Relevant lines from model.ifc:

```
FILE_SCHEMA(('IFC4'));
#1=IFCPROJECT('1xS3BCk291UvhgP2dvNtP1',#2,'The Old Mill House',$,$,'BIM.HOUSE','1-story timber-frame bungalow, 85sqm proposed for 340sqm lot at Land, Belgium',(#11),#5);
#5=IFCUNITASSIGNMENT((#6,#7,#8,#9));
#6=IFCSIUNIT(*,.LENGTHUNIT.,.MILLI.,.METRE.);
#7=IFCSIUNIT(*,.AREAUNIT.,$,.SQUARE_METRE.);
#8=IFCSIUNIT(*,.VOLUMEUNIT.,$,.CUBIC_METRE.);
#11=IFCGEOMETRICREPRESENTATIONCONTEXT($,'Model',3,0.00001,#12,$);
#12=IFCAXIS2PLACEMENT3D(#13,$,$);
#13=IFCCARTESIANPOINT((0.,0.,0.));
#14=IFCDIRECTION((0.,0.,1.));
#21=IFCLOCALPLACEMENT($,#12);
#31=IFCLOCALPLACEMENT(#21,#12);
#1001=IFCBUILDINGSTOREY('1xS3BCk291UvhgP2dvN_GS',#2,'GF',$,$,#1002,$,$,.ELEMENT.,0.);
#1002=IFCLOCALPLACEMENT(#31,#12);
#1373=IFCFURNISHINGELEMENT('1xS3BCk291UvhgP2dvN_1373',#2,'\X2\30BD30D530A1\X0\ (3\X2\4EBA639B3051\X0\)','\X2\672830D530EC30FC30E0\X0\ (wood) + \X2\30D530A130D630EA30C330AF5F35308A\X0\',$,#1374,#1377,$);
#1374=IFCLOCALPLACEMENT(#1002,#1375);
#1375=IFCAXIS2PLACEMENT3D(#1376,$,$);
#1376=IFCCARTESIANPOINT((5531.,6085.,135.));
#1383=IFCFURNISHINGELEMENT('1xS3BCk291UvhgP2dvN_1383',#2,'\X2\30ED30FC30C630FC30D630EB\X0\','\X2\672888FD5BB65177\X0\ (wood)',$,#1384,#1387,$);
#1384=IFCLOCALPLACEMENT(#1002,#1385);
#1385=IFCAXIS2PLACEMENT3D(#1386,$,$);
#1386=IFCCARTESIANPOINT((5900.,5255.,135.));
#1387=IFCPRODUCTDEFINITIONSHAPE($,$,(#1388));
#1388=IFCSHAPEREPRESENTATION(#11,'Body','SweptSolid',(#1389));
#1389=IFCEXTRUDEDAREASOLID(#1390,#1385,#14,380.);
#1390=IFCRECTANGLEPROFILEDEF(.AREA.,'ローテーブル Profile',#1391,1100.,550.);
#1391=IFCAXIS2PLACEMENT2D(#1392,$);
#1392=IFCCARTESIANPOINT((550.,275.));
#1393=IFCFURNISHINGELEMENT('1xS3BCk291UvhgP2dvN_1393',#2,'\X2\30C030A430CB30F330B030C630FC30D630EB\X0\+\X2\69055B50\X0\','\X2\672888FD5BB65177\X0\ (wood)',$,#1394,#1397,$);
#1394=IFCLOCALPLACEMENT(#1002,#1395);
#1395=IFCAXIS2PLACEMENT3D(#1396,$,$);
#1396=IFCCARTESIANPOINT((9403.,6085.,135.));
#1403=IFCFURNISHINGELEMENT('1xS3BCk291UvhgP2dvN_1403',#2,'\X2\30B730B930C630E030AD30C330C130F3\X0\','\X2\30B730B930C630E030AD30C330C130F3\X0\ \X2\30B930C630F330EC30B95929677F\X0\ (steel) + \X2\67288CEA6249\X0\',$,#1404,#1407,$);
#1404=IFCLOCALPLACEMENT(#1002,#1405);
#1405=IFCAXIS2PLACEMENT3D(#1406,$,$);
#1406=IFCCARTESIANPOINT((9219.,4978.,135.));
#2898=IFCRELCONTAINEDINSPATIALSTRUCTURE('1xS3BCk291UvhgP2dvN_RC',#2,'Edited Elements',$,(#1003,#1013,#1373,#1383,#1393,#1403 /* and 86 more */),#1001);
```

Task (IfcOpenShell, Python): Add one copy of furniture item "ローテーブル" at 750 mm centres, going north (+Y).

```python
import numpy as np
import ifcopenshell
import ifcopenshell.api.geometry
import ifcopenshell.api.root
import ifcopenshell.util.element
import ifcopenshell.util.placement
import ifcopenshell.util.unit

model = ifcopenshell.open("model.ifc")
unit_scale = ifcopenshell.util.unit.calculate_unit_scale(model)


def reuse_history(source, copy):
    """copy_class also copies each property set's owner history, people and application; keep the originals."""
    for rel in copy.IsDefinedBy:
        if rel.is_a("IfcRelDefinesByProperties") and (history := rel.RelatingPropertyDefinition.OwnerHistory):
            rel.RelatingPropertyDefinition.OwnerHistory = source.OwnerHistory
            ifcopenshell.util.element.remove_deep2(model, history)


source = model.by_guid("1xS3BCk291UvhgP2dvN_1383")
base = ifcopenshell.util.placement.get_local_placement(source.ObjectPlacement)
step = np.array([0.0, 1.0, 0.0]) * 0.75 / unit_scale

for i in range(1, 2):
    copy = ifcopenshell.api.root.copy_class(model, product=source)
    copy.Representation = ifcopenshell.util.element.copy_deep(
        model, source.Representation, exclude=["IfcGeometricRepresentationContext", "IfcRepresentationMap"]
    )
    reuse_history(source, copy)
    matrix = base.copy()
    matrix[:3, 3] += i * step
    print("added at", matrix[:3, 3].round(3) + 0.0)
    ifcopenshell.api.geometry.edit_object_placement(model, product=copy, matrix=matrix, is_si=False)

model.write("model_edited.ifc")
```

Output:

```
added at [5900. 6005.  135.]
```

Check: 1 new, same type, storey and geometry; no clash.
